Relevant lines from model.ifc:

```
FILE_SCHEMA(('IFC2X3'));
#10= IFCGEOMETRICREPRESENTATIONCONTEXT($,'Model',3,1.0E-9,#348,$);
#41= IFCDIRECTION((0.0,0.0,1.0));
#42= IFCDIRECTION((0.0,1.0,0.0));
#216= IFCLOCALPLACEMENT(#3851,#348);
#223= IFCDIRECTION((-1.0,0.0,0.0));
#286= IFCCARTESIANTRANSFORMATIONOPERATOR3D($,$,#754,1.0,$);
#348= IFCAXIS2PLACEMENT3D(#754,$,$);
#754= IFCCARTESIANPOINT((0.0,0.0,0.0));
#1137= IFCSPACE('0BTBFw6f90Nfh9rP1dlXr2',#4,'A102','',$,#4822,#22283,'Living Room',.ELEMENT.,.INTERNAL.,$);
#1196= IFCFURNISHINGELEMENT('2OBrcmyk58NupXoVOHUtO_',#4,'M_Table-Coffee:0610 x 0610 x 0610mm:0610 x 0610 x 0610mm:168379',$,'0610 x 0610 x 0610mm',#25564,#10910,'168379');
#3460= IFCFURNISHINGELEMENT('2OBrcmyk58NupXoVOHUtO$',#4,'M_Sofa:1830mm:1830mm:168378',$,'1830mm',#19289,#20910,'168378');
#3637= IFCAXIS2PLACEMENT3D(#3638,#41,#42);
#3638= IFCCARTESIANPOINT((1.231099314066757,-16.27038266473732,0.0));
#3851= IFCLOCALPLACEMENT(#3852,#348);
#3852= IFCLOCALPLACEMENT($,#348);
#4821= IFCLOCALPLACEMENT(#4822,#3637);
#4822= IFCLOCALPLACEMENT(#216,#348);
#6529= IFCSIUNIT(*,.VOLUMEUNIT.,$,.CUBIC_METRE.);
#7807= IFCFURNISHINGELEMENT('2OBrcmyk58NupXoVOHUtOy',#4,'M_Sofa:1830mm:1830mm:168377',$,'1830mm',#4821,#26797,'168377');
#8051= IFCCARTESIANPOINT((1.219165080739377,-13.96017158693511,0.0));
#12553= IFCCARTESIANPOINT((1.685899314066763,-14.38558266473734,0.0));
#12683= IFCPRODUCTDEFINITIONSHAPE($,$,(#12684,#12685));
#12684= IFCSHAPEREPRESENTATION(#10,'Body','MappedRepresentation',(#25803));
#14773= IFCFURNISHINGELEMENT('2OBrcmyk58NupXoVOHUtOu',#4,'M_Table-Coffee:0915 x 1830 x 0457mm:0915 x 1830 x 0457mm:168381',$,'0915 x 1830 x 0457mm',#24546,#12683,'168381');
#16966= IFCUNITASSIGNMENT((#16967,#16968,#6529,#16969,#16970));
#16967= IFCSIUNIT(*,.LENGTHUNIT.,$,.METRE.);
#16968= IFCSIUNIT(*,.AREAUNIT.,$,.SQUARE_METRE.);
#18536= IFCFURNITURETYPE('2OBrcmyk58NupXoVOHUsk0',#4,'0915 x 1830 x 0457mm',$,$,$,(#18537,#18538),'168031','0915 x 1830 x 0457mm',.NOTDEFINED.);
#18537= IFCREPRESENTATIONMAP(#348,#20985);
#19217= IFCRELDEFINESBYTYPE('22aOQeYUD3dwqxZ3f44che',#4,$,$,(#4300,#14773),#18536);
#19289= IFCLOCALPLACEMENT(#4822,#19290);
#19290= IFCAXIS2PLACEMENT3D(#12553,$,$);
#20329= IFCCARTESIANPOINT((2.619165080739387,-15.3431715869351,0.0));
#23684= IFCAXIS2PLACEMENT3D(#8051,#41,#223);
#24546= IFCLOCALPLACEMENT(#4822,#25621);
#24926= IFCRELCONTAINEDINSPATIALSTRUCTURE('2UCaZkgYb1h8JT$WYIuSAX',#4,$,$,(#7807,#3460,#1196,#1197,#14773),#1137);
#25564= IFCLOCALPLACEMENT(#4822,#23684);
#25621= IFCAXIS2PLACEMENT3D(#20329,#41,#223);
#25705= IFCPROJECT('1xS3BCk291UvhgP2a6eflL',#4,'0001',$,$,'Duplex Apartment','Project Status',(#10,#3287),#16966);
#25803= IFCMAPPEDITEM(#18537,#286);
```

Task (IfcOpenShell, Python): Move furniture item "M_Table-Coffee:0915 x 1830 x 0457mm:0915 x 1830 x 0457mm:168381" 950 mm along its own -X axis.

```python
import ifcopenshell
import ifcopenshell.api.geometry
import ifcopenshell.util.placement

model = ifcopenshell.open("model.ifc")

item = model.by_guid("2OBrcmyk58NupXoVOHUtOu")
matrix = ifcopenshell.util.placement.get_local_placement(item.ObjectPlacement)
matrix[:3, 3] -= matrix[:3, 0] * 0.95
ifcopenshell.api.geometry.edit_object_placement(model, product=item, matrix=matrix, is_si=False)

print(ifcopenshell.util.placement.get_local_placement(item.ObjectPlacement).round(3) + 0.0)

model.write("model-out.ifc")
```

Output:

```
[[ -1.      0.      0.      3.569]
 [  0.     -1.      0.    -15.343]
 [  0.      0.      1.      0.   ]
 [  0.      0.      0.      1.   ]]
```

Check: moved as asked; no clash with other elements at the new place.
